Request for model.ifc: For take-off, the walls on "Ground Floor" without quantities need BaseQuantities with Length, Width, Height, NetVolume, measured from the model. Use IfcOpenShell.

First a look at what the model holds.

```python
import ifcopenshell
import ifcopenshell.util.element
import ifcopenshell.util.unit

model = ifcopenshell.open("model.ifc")
print(model.schema)
for unit_type in ("LENGTHUNIT", "AREAUNIT", "VOLUMEUNIT"):
    print(unit_type, ifcopenshell.util.unit.calculate_unit_scale(model, unit_type))
storey = next(s for s in model.by_type("IfcBuildingStorey") if s.Name == "Ground Floor")
walls = [e for e in ifcopenshell.util.element.get_decomposition(storey) if e.is_a("IfcWall")]
for e in sorted(walls, key=lambda e: e.id()):
    print(e.id(), e.is_a(), e.Name, list(ifcopenshell.util.element.get_psets(e, qtos_only=True)), sep=" | ")
```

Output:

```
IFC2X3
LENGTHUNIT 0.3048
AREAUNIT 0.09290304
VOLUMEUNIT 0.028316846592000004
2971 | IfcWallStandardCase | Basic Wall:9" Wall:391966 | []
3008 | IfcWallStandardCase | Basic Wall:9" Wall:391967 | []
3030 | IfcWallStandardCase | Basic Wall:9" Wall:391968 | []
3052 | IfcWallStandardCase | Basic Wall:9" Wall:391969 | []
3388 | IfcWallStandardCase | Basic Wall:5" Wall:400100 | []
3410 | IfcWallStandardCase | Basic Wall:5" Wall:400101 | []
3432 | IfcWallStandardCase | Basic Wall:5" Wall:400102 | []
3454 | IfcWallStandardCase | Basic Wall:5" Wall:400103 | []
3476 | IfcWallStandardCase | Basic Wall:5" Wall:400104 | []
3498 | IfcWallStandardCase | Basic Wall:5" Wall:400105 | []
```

```python
import ifcopenshell
import ifcopenshell.api.pset
import ifcopenshell.geom
import ifcopenshell.util.element
import ifcopenshell.util.shape
import ifcopenshell.util.unit

model = ifcopenshell.open("model.ifc")
unit_scale = ifcopenshell.util.unit.calculate_unit_scale(model)
volume_scale = ifcopenshell.util.unit.calculate_unit_scale(model, "VOLUMEUNIT")
settings = ifcopenshell.geom.settings()

storey = next(s for s in model.by_type("IfcBuildingStorey") if s.Name == "Ground Floor")
walls = [e for e in ifcopenshell.util.element.get_decomposition(storey) if e.is_a("IfcWall")]

for e in sorted(walls, key=lambda e: e.id()):
    if ifcopenshell.util.element.get_psets(e, qtos_only=True, should_inherit=False):
        continue
    # Geometry comes back in metres, in the element's own axes.
    shape = ifcopenshell.geom.create_shape(settings, e)
    values = {
        "Length": ifcopenshell.util.shape.get_x(shape.geometry) / unit_scale,
        "Width": ifcopenshell.util.shape.get_y(shape.geometry) / unit_scale,
        "Height": ifcopenshell.util.shape.get_z(shape.geometry) / unit_scale,
        "NetVolume": ifcopenshell.util.shape.get_volume(shape.geometry) / volume_scale,
    }
    qto = ifcopenshell.api.pset.add_qto(model, product=e, name="BaseQuantities")
    ifcopenshell.api.pset.edit_qto(model, qto=qto, properties=values)
    print(e.id(), {k: round(v, 3) for k, v in values.items()})

model.write("model_edited.ifc")
```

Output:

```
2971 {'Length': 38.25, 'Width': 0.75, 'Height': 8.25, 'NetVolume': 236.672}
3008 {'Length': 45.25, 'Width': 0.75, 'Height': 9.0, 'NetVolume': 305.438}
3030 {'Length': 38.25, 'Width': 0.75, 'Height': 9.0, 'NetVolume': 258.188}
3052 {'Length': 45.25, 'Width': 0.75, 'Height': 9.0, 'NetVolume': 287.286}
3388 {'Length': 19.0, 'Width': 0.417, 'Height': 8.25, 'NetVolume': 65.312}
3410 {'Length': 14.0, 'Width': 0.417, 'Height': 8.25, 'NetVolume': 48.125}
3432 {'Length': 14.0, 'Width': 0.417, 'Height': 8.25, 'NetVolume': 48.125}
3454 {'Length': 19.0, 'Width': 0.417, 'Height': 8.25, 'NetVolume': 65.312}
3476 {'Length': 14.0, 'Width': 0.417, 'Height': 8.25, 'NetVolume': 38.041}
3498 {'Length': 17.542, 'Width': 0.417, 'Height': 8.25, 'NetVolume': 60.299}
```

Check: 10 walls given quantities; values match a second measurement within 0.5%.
